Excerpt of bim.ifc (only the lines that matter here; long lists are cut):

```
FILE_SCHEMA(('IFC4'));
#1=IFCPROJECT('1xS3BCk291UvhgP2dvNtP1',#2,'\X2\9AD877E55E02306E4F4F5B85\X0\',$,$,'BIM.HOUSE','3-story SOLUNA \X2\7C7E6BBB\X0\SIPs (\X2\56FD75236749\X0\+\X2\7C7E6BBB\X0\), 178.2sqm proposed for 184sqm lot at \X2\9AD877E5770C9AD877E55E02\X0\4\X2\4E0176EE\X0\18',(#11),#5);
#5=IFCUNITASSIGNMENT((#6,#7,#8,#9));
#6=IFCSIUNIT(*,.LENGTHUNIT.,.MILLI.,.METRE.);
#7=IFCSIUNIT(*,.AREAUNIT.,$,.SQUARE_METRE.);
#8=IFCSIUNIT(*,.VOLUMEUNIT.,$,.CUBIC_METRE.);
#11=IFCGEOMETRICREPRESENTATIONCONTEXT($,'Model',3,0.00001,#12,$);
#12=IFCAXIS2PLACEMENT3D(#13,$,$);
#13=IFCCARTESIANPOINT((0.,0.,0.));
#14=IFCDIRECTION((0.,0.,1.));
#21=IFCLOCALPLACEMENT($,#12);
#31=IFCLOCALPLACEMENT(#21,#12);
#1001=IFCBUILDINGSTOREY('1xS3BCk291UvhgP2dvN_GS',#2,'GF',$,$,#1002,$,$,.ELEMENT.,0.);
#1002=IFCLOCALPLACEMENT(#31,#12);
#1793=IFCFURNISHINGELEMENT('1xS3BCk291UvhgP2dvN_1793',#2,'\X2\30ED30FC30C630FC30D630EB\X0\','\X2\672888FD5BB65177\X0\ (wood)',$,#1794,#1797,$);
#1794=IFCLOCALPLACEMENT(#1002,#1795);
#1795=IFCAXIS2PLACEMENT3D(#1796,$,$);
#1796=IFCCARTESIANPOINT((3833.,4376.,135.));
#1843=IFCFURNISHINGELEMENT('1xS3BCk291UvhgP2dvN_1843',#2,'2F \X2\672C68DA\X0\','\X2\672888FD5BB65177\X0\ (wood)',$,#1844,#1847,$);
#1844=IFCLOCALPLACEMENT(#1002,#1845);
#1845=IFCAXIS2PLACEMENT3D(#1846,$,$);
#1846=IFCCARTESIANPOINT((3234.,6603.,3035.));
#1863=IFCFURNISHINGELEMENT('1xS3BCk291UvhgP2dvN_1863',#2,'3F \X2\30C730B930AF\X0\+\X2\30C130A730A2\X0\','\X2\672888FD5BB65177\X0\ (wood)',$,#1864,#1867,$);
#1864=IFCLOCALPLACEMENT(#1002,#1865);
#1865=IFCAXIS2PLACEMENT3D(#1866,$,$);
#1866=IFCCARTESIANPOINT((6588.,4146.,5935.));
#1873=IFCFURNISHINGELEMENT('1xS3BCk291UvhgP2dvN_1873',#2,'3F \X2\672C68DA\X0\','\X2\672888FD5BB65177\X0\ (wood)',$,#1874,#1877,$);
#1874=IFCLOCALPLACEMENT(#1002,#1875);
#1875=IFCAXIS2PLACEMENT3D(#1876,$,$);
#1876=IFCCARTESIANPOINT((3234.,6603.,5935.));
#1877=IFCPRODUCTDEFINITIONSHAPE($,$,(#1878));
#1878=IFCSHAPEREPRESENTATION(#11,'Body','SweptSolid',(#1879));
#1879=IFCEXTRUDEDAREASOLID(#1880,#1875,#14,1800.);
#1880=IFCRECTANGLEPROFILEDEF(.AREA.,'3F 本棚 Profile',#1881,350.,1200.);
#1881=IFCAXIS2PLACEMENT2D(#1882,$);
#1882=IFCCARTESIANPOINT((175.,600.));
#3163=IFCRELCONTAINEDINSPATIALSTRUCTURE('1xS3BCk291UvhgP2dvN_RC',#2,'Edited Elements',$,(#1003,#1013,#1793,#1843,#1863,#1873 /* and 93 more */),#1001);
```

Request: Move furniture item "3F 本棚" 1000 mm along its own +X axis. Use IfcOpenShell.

```python
import ifcopenshell
import ifcopenshell.api.geometry
import ifcopenshell.util.placement
import ifcopenshell.util.unit

model = ifcopenshell.open("bim.ifc")
unit_scale = ifcopenshell.util.unit.calculate_unit_scale(model)

item = model.by_guid("1xS3BCk291UvhgP2dvN_1873")
matrix = ifcopenshell.util.placement.get_local_placement(item.ObjectPlacement)
matrix[:3, 3] += matrix[:3, 0] * 1 / unit_scale
ifcopenshell.api.geometry.edit_object_placement(model, product=item, matrix=matrix, is_si=False)

print(ifcopenshell.util.placement.get_local_placement(item.ObjectPlacement).round(3) + 0.0)

model.write("bim-out.ifc")
```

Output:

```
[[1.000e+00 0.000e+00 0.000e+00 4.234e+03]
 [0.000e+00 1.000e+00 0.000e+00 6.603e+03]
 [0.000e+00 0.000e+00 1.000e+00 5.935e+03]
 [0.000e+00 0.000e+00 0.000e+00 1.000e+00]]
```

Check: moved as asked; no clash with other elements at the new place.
